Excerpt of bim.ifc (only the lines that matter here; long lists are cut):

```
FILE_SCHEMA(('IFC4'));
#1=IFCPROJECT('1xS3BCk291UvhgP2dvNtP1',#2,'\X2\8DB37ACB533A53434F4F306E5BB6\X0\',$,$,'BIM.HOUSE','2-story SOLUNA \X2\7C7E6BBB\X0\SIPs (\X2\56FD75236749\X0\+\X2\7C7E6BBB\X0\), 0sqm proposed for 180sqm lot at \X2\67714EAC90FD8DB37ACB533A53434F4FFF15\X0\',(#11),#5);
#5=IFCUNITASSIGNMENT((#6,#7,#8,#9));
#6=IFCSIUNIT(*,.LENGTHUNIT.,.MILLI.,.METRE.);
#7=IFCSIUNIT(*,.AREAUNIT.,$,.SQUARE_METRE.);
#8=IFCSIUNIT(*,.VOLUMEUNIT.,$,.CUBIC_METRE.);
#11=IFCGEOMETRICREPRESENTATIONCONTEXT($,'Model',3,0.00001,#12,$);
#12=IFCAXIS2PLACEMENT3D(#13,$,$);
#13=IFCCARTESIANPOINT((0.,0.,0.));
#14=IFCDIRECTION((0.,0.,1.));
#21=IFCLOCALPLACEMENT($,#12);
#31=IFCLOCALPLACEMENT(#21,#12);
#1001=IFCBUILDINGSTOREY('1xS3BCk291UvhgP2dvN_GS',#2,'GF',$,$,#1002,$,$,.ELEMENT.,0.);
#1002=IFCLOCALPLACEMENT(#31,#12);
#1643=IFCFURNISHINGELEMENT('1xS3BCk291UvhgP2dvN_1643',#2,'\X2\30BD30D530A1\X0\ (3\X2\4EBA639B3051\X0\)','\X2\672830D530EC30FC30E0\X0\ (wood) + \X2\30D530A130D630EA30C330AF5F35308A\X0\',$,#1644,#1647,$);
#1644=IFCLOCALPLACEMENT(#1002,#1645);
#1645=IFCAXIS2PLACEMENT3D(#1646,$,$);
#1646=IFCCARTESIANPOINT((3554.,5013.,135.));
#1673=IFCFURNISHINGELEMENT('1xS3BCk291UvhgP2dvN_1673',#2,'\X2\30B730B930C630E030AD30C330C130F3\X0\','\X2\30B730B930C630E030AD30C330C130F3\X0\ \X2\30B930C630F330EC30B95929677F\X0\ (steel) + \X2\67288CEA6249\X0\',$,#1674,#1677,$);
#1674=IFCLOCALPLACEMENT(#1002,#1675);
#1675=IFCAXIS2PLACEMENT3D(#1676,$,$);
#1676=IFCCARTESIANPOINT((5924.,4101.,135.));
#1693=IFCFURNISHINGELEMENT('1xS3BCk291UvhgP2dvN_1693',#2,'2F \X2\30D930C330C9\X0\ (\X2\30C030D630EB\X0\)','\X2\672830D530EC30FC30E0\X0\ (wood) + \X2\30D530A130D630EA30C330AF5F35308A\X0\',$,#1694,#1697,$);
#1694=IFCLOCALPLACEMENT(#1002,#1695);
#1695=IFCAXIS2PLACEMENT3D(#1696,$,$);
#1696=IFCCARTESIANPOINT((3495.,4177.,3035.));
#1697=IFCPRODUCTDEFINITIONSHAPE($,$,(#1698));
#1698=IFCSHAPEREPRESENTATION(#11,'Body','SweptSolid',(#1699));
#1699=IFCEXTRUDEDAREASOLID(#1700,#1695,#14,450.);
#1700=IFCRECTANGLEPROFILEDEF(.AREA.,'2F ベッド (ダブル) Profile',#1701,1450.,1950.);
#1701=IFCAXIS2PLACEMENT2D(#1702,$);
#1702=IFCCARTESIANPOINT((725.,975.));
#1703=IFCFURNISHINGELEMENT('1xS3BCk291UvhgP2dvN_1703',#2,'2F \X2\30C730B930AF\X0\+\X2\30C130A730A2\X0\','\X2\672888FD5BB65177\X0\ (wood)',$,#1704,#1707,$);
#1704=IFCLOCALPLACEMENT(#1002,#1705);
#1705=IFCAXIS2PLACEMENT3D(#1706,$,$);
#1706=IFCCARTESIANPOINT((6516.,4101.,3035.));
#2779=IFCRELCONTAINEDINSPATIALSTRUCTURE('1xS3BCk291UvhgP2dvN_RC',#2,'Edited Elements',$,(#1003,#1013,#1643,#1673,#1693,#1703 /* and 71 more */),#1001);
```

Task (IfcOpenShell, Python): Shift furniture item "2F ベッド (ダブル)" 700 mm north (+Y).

```python
import ifcopenshell
import ifcopenshell.api.geometry
import ifcopenshell.util.placement
import ifcopenshell.util.unit

model = ifcopenshell.open("bim.ifc")
unit_scale = ifcopenshell.util.unit.calculate_unit_scale(model)

item = model.by_guid("1xS3BCk291UvhgP2dvN_1693")
matrix = ifcopenshell.util.placement.get_local_placement(item.ObjectPlacement)
matrix[1, 3] += 0.7 / unit_scale
ifcopenshell.api.geometry.edit_object_placement(model, product=item, matrix=matrix, is_si=False)

print(ifcopenshell.util.placement.get_local_placement(item.ObjectPlacement).round(3) + 0.0)

model.write("bim_updated.ifc")
```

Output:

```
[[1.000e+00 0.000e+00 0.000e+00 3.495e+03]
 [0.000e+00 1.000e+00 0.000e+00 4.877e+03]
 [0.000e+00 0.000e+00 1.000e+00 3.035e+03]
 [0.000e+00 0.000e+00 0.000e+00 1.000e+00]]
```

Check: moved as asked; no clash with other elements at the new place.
